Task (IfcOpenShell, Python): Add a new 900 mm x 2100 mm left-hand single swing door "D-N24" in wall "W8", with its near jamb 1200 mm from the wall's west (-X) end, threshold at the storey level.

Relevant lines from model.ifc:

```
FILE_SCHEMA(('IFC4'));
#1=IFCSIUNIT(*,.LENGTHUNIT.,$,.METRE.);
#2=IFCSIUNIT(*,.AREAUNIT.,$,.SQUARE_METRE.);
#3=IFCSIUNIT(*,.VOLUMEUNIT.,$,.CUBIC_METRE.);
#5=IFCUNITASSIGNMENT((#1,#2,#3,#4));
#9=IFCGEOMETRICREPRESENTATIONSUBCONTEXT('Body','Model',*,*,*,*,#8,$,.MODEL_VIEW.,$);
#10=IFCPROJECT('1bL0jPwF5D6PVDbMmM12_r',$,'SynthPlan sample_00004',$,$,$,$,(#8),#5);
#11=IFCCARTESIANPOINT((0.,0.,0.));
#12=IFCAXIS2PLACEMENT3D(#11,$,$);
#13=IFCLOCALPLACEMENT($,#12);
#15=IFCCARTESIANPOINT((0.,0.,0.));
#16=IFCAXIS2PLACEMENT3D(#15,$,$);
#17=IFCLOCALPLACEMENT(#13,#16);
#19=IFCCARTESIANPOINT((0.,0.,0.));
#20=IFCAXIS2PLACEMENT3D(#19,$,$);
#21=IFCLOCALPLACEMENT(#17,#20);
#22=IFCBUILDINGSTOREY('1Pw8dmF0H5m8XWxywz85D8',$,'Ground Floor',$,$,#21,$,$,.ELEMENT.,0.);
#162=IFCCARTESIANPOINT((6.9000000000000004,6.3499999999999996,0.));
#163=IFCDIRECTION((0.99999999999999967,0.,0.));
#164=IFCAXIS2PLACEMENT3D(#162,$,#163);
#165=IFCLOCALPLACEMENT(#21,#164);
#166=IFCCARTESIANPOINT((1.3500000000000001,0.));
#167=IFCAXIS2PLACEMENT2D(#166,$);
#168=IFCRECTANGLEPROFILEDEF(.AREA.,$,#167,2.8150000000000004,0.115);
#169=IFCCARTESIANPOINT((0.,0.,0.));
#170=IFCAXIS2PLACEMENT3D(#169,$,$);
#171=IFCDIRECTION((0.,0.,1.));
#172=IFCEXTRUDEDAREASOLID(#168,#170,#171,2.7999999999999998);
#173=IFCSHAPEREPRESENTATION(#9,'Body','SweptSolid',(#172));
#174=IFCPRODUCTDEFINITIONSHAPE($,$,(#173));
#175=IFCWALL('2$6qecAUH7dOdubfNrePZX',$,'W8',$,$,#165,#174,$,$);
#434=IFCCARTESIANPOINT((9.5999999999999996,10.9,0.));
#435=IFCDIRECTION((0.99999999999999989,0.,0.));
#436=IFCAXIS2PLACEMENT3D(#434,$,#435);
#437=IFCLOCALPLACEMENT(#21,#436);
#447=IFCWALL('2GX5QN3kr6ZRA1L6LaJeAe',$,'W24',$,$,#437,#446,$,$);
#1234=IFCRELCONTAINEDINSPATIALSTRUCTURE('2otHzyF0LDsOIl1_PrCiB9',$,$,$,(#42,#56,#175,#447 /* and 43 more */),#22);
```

```python
import numpy as np
import ifcopenshell
import ifcopenshell.api.feature
import ifcopenshell.api.geometry
import ifcopenshell.api.root
import ifcopenshell.api.spatial
import ifcopenshell.geom
import ifcopenshell.util.element
import ifcopenshell.util.placement
import ifcopenshell.util.representation
import ifcopenshell.util.shape
import ifcopenshell.util.unit

model = ifcopenshell.open("model.ifc")
unit_scale = ifcopenshell.util.unit.calculate_unit_scale(model)
settings = ifcopenshell.geom.settings()


def volume(element):
    """Net volume in cubic metres, openings subtracted."""
    shape = ifcopenshell.geom.create_shape(settings, element)
    return ifcopenshell.util.shape.get_volume(shape.geometry)


wall = model.by_guid("2$6qecAUH7dOdubfNrePZX")
storey = ifcopenshell.util.element.get_container(wall, ifc_class="IfcBuildingStorey")
context = ifcopenshell.util.representation.get_context(model, "Model", "Body", "MODEL_VIEW")
before = volume(wall)

width, height, from_end, sill = 0.9, 2.1, 1.2, 0.0  # metres

# The wall runs along its own X axis, and the end named is its -X end.
wall_shape = ifcopenshell.geom.create_shape(settings, wall)
x, y, z = ifcopenshell.util.shape.get_vertices(wall_shape.geometry).T
start = x.min() + from_end
face, thickness = float(y.min()), float(y.max() - y.min())
wall_matrix = ifcopenshell.util.placement.get_local_placement(wall.ObjectPlacement)
level = ifcopenshell.util.placement.get_local_placement(storey.ObjectPlacement)[2, 3]


def in_wall(x, y):
    """Placement at x, y metres in the wall's axes, at sill height."""
    matrix = wall_matrix.copy()
    matrix[:, 3] = wall_matrix @ np.array([x / unit_scale, y / unit_scale, 0.0, 1.0])
    matrix[2, 3] = level + sill / unit_scale
    return matrix


# Opening: a box that overshoots both wall faces by 50 mm.
opening = ifcopenshell.api.root.create_entity(model, ifc_class="IfcOpeningElement", predefined_type="OPENING")
box = ifcopenshell.api.geometry.add_wall_representation(
    model, context=context, length=width, height=height, thickness=thickness + 0.1
)
ifcopenshell.api.geometry.assign_representation(model, product=opening, representation=box)
ifcopenshell.api.geometry.edit_object_placement(model, product=opening, matrix=in_wall(start, face - 0.05), is_si=False)
ifcopenshell.api.feature.add_feature(model, feature=opening, element=wall)

door = ifcopenshell.api.root.create_entity(model, ifc_class="IfcDoor", name="D-N24", predefined_type="DOOR")
door.OverallWidth, door.OverallHeight = width / unit_scale, height / unit_scale
door.OperationType = "SINGLE_SWING_LEFT"
body = ifcopenshell.api.geometry.add_door_representation(
    model,
    context=context,
    overall_width=door.OverallWidth,
    overall_height=door.OverallHeight,
    operation_type="SINGLE_SWING_LEFT",
    lining_properties={"LiningDepth": thickness / unit_scale, "ThresholdDepth": thickness / unit_scale},
)
ifcopenshell.api.geometry.assign_representation(model, product=door, representation=body)
ifcopenshell.api.spatial.assign_container(model, products=[door], relating_structure=storey)
ifcopenshell.api.feature.add_filling(model, opening=opening, element=door)

# The lining spans the wall, so the door starts at the wall face.
ifcopenshell.api.geometry.edit_object_placement(model, product=door, matrix=in_wall(start, face), is_si=False)

after = volume(wall)

print(f"wall volume {before:.3f} -> {after:.3f} m3")

model.write("model_rev.ifc")
```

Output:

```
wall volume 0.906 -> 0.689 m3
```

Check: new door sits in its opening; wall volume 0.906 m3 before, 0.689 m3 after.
